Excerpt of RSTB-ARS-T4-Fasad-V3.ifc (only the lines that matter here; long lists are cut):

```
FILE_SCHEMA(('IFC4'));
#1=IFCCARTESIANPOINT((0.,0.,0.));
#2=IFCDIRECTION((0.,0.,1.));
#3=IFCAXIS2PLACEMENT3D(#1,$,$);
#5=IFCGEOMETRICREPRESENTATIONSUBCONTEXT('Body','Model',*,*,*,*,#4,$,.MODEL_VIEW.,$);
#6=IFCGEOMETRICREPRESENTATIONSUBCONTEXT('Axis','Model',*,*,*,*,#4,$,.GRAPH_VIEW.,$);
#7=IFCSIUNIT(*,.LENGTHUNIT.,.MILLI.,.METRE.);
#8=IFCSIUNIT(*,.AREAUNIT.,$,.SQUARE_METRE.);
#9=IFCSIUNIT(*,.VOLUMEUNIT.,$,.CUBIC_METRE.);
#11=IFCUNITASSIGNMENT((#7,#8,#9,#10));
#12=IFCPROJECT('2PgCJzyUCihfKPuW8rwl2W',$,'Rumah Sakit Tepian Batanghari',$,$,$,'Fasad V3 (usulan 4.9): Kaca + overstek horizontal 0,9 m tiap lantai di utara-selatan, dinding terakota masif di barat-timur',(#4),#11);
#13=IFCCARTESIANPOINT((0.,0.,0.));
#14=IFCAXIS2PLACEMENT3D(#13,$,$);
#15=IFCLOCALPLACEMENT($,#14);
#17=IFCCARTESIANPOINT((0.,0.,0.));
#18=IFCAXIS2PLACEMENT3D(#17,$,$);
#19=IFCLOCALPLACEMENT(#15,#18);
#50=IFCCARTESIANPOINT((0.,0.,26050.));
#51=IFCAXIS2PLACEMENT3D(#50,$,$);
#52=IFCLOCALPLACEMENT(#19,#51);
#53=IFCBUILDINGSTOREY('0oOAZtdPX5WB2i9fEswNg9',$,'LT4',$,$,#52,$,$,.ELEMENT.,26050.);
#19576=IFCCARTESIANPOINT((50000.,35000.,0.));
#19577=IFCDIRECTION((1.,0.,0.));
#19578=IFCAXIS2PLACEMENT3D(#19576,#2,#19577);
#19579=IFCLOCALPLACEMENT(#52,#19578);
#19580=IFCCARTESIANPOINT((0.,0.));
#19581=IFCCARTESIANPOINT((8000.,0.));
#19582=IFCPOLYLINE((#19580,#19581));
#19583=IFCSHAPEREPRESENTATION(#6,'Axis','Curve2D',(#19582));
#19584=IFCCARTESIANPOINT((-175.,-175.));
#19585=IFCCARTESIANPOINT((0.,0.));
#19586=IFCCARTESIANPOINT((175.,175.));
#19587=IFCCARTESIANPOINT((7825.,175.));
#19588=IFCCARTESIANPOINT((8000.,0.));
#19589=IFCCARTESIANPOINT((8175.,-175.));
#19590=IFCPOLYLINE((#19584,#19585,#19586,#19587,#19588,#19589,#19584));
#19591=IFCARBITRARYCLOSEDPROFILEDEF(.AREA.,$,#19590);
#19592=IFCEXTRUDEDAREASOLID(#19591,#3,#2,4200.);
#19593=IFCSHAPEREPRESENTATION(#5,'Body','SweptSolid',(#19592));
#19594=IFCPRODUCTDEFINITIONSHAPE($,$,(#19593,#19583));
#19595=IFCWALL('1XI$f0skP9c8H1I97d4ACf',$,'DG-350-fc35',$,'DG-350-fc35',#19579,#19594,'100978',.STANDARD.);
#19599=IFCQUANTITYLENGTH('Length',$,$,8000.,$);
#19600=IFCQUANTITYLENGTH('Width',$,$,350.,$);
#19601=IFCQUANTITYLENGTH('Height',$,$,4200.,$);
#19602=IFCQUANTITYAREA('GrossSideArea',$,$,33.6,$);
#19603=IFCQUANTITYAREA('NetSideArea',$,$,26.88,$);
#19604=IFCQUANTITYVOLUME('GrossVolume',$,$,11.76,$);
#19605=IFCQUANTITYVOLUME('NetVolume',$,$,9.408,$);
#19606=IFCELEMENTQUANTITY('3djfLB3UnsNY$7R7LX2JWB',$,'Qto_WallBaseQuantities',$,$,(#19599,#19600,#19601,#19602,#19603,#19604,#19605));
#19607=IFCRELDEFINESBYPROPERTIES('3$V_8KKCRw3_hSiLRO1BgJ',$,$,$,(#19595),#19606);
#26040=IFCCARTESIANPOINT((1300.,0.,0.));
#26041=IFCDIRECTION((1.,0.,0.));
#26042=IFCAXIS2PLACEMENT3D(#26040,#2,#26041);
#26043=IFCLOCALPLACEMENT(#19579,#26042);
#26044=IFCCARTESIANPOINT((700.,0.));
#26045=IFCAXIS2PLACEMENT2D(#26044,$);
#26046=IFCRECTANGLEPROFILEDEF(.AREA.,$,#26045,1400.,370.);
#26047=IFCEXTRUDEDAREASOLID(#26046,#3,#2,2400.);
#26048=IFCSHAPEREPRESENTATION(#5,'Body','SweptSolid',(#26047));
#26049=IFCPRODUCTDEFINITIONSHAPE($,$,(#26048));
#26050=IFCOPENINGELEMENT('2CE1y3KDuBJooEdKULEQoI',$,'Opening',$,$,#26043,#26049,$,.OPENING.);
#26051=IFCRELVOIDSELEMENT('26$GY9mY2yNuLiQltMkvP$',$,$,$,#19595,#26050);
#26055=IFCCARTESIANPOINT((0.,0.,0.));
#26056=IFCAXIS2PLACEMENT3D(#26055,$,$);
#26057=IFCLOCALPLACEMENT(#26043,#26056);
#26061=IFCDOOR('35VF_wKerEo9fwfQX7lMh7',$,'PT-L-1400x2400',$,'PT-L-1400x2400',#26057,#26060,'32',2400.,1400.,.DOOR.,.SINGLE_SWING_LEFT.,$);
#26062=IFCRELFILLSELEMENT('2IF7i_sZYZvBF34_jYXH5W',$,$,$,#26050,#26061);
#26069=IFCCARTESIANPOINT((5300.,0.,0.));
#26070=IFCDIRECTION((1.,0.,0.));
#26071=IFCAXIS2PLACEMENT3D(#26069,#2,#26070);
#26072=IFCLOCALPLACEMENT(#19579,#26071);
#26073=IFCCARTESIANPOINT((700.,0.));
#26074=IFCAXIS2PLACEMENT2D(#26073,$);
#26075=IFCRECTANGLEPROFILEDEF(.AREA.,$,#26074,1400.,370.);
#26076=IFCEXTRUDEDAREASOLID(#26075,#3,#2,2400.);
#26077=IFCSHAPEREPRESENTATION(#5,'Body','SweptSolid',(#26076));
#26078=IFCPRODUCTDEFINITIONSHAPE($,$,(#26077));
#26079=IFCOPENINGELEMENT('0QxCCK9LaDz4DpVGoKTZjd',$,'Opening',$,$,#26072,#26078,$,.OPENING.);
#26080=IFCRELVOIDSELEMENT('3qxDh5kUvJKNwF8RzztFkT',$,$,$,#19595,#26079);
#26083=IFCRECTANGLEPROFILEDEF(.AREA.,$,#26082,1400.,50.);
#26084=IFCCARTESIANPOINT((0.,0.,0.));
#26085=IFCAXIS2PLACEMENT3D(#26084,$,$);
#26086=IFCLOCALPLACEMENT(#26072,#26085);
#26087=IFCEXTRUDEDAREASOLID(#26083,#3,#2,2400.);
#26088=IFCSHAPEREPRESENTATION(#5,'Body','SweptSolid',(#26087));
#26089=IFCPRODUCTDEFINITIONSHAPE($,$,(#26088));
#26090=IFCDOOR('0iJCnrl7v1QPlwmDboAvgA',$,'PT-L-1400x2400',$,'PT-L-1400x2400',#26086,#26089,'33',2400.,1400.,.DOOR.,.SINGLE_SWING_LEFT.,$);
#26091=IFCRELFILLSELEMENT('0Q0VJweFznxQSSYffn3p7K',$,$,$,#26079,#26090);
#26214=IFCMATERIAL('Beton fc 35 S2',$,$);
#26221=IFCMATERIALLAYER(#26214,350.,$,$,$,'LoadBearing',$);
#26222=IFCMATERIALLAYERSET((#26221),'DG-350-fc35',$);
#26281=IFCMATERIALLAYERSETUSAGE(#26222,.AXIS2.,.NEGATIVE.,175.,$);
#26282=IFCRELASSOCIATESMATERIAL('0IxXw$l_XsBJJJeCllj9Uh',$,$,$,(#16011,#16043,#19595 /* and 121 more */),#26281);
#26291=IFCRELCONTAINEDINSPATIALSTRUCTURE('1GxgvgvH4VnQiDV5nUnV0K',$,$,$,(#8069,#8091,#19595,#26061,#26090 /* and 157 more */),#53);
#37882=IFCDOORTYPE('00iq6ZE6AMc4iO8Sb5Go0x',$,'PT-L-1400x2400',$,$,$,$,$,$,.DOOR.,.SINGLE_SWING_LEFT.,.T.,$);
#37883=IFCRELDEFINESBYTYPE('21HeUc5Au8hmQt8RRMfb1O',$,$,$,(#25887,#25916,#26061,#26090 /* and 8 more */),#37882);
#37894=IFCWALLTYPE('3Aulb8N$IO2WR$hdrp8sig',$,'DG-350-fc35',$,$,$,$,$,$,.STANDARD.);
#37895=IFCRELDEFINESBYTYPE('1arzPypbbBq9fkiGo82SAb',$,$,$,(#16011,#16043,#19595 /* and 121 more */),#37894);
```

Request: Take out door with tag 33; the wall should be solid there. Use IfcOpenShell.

```python
import ifcopenshell
import ifcopenshell.api.feature
import ifcopenshell.api.pset
import ifcopenshell.api.root
import ifcopenshell.geom
import ifcopenshell.util.element
import ifcopenshell.util.shape
import ifcopenshell.util.unit

model = ifcopenshell.open("RSTB-ARS-T4-Fasad-V3.ifc")
area_scale = ifcopenshell.util.unit.calculate_unit_scale(model, "AREAUNIT")
volume_scale = ifcopenshell.util.unit.calculate_unit_scale(model, "VOLUMEUNIT")
settings = ifcopenshell.geom.settings()


def volume(element):
    """Net volume in cubic metres, openings subtracted."""
    shape = ifcopenshell.geom.create_shape(settings, element)
    return ifcopenshell.util.shape.get_volume(shape.geometry)


door = model.by_guid("0iJCnrl7v1QPlwmDboAvgA")
opening = door.FillsVoids[0].RelatingOpeningElement
wall = opening.VoidsElements[0].RelatingBuildingElement
before = volume(wall)

ifcopenshell.api.root.remove_product(model, product=door)
ifcopenshell.api.feature.remove_feature(model, feature=opening)

after = volume(wall)
thickness = 0.35  # wall thickness in metres

# Update the wall's stored quantities.
qto = model.by_id(ifcopenshell.util.element.get_pset(wall, "Qto_WallBaseQuantities", should_inherit=False)["id"])
ifcopenshell.api.pset.edit_qto(model, qto=qto, properties={
    "NetSideArea": after / thickness / area_scale,
    "NetVolume": after / volume_scale,
})

print(f"wall volume {before:.3f} -> {after:.3f} m3")

model.write("RSTB-ARS-T4-Fasad-V3_rev.ifc")
```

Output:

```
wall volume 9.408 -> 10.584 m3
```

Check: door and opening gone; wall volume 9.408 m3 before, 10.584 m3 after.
